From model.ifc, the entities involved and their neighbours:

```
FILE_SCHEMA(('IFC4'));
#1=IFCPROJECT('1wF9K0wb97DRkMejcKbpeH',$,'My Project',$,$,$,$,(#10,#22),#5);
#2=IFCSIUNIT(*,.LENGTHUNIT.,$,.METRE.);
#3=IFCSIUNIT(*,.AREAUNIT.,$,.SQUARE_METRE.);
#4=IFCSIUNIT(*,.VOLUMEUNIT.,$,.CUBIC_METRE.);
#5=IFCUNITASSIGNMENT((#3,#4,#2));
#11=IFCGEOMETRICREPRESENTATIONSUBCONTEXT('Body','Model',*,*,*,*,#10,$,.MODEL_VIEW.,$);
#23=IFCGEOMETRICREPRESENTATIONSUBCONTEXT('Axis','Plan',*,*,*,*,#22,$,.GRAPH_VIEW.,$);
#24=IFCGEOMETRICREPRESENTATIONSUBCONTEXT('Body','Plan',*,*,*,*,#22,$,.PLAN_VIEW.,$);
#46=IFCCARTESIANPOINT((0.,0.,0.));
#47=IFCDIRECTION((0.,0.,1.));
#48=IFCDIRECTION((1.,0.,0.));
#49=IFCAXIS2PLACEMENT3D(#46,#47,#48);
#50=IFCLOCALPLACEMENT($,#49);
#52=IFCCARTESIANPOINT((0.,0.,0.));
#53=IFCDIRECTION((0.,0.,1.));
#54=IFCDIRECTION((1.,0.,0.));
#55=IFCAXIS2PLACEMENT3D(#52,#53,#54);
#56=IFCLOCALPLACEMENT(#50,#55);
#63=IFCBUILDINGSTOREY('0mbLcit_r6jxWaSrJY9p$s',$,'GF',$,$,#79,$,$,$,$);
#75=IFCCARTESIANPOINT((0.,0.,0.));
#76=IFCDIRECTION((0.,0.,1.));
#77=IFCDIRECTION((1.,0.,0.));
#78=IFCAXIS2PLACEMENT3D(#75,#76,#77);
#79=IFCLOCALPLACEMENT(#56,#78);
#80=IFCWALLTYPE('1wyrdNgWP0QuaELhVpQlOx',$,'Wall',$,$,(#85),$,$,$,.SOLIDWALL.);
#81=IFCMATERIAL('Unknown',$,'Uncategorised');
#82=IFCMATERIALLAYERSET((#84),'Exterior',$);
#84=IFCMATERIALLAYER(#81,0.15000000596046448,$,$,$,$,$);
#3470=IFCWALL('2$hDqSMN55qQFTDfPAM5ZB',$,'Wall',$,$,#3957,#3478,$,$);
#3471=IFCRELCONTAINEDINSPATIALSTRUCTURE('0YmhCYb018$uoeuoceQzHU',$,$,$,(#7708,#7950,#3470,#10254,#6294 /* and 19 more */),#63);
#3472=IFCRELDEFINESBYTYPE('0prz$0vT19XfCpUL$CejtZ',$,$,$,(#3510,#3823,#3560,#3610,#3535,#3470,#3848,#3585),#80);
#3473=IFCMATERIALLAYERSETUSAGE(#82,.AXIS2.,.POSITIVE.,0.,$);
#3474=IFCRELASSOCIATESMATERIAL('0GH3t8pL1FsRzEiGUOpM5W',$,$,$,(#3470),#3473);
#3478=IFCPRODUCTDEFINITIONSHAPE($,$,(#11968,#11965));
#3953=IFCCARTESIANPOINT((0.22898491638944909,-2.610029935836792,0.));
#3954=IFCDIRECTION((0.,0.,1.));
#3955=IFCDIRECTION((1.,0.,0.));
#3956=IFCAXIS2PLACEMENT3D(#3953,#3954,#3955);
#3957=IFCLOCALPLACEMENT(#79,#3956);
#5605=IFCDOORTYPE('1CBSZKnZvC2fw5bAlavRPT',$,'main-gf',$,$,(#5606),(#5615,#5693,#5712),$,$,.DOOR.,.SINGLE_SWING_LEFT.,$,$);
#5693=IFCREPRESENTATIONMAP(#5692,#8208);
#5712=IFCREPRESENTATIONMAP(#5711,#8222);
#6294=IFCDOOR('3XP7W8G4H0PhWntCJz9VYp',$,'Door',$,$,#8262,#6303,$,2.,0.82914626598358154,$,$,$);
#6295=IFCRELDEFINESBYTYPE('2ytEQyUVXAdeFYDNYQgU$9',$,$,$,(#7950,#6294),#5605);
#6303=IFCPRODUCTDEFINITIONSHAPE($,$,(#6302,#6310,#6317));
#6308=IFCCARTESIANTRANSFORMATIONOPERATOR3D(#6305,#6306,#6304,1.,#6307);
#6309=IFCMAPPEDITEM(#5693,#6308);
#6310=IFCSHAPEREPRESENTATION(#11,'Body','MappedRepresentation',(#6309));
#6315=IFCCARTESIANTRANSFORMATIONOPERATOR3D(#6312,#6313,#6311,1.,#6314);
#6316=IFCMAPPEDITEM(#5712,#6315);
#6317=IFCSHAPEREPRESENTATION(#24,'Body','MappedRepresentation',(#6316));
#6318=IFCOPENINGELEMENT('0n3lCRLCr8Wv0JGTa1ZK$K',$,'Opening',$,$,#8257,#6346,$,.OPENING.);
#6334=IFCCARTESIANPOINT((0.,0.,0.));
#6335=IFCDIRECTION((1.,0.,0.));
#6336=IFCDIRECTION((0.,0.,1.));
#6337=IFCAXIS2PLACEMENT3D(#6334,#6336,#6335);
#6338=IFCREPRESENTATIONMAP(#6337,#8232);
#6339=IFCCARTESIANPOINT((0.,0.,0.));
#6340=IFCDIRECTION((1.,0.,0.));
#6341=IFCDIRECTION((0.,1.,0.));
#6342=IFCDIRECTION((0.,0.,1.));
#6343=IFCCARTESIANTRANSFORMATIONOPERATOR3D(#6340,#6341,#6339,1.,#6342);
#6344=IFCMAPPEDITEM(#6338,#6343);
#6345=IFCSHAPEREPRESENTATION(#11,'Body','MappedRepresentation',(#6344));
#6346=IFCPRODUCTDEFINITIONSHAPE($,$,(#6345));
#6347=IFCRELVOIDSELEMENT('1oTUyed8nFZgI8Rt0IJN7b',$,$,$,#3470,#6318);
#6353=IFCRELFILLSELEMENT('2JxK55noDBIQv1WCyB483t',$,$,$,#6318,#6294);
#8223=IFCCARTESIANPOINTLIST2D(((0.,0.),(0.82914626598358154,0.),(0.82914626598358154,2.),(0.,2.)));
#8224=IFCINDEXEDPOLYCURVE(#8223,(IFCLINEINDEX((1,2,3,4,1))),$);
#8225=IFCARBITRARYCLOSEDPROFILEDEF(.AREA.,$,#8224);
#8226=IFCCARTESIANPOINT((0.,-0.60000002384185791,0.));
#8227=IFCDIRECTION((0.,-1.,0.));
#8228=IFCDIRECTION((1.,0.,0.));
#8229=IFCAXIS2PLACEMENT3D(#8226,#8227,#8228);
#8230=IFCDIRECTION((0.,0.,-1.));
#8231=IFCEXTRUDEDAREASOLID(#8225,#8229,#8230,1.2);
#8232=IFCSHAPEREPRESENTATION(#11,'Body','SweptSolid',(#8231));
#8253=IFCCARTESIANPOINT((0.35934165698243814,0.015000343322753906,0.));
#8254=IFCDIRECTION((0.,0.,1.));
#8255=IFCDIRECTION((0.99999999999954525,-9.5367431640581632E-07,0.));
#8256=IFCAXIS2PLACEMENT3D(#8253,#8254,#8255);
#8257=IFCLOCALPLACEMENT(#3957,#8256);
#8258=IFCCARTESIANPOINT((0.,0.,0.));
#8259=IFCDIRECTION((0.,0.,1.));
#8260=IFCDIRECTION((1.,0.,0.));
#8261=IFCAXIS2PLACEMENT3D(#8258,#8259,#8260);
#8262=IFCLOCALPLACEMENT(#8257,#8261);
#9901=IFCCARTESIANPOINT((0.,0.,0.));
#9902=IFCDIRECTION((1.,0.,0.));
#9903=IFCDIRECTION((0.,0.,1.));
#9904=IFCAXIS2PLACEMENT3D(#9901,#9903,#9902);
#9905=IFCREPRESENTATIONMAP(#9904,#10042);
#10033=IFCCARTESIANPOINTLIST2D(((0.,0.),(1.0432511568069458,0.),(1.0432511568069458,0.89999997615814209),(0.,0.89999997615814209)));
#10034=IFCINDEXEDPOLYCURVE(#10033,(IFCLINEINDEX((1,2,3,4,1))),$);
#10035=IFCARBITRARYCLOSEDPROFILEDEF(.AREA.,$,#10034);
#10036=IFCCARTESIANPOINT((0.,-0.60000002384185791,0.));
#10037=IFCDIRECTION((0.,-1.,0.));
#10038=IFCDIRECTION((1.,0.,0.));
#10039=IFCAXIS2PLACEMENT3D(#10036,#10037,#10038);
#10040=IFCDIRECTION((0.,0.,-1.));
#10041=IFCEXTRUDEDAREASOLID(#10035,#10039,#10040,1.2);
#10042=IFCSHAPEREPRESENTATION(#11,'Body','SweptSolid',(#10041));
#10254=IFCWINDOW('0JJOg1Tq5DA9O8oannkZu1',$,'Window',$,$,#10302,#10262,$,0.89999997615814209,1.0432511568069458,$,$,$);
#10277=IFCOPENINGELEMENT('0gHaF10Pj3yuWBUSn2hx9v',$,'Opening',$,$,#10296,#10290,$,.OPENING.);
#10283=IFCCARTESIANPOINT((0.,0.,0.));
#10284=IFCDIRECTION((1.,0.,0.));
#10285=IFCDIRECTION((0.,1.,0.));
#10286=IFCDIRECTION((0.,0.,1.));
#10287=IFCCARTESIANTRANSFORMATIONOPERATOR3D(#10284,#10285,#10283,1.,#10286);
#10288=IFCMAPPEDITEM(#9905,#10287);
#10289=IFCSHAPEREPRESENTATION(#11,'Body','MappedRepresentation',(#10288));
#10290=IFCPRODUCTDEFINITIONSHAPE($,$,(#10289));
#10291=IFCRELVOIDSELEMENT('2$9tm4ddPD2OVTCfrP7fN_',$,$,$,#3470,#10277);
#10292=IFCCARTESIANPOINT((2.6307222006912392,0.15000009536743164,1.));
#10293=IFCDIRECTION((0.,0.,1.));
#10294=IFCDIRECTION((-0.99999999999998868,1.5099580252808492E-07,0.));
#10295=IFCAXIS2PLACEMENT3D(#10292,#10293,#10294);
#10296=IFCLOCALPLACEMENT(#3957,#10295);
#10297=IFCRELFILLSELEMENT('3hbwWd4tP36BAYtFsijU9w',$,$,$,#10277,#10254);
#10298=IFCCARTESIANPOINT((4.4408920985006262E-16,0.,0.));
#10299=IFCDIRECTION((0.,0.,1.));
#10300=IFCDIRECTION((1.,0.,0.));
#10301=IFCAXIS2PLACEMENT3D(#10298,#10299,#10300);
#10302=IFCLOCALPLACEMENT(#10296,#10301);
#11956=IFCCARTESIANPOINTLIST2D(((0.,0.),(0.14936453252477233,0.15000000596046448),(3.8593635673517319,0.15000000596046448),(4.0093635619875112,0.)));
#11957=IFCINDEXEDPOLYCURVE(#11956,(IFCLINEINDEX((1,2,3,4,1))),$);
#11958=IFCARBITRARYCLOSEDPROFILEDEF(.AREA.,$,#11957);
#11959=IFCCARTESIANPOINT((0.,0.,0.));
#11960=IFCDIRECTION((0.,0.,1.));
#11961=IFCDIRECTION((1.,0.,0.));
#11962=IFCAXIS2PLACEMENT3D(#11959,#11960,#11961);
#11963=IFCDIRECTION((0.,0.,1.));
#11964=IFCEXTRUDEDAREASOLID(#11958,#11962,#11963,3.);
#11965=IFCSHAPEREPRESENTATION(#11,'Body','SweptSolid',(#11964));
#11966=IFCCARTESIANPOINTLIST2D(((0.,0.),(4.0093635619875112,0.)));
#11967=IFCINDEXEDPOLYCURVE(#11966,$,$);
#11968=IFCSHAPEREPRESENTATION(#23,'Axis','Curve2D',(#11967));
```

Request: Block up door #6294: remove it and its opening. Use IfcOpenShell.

```python
import ifcopenshell
import ifcopenshell.api.feature
import ifcopenshell.api.root
import ifcopenshell.geom
import ifcopenshell.util.shape

model = ifcopenshell.open("model.ifc")
settings = ifcopenshell.geom.settings()


def volume(element):
    """Net volume in cubic metres, openings subtracted."""
    shape = ifcopenshell.geom.create_shape(settings, element)
    return ifcopenshell.util.shape.get_volume(shape.geometry)


door = model.by_guid("3XP7W8G4H0PhWntCJz9VYp")
opening = door.FillsVoids[0].RelatingOpeningElement
wall = opening.VoidsElements[0].RelatingBuildingElement
before = volume(wall)

ifcopenshell.api.root.remove_product(model, product=door)
ifcopenshell.api.feature.remove_feature(model, feature=opening)

after = volume(wall)

print(f"wall volume {before:.3f} -> {after:.3f} m3")

model.write("model_updated.ifc")
```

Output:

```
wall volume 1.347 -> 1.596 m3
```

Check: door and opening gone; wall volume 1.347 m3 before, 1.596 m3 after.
